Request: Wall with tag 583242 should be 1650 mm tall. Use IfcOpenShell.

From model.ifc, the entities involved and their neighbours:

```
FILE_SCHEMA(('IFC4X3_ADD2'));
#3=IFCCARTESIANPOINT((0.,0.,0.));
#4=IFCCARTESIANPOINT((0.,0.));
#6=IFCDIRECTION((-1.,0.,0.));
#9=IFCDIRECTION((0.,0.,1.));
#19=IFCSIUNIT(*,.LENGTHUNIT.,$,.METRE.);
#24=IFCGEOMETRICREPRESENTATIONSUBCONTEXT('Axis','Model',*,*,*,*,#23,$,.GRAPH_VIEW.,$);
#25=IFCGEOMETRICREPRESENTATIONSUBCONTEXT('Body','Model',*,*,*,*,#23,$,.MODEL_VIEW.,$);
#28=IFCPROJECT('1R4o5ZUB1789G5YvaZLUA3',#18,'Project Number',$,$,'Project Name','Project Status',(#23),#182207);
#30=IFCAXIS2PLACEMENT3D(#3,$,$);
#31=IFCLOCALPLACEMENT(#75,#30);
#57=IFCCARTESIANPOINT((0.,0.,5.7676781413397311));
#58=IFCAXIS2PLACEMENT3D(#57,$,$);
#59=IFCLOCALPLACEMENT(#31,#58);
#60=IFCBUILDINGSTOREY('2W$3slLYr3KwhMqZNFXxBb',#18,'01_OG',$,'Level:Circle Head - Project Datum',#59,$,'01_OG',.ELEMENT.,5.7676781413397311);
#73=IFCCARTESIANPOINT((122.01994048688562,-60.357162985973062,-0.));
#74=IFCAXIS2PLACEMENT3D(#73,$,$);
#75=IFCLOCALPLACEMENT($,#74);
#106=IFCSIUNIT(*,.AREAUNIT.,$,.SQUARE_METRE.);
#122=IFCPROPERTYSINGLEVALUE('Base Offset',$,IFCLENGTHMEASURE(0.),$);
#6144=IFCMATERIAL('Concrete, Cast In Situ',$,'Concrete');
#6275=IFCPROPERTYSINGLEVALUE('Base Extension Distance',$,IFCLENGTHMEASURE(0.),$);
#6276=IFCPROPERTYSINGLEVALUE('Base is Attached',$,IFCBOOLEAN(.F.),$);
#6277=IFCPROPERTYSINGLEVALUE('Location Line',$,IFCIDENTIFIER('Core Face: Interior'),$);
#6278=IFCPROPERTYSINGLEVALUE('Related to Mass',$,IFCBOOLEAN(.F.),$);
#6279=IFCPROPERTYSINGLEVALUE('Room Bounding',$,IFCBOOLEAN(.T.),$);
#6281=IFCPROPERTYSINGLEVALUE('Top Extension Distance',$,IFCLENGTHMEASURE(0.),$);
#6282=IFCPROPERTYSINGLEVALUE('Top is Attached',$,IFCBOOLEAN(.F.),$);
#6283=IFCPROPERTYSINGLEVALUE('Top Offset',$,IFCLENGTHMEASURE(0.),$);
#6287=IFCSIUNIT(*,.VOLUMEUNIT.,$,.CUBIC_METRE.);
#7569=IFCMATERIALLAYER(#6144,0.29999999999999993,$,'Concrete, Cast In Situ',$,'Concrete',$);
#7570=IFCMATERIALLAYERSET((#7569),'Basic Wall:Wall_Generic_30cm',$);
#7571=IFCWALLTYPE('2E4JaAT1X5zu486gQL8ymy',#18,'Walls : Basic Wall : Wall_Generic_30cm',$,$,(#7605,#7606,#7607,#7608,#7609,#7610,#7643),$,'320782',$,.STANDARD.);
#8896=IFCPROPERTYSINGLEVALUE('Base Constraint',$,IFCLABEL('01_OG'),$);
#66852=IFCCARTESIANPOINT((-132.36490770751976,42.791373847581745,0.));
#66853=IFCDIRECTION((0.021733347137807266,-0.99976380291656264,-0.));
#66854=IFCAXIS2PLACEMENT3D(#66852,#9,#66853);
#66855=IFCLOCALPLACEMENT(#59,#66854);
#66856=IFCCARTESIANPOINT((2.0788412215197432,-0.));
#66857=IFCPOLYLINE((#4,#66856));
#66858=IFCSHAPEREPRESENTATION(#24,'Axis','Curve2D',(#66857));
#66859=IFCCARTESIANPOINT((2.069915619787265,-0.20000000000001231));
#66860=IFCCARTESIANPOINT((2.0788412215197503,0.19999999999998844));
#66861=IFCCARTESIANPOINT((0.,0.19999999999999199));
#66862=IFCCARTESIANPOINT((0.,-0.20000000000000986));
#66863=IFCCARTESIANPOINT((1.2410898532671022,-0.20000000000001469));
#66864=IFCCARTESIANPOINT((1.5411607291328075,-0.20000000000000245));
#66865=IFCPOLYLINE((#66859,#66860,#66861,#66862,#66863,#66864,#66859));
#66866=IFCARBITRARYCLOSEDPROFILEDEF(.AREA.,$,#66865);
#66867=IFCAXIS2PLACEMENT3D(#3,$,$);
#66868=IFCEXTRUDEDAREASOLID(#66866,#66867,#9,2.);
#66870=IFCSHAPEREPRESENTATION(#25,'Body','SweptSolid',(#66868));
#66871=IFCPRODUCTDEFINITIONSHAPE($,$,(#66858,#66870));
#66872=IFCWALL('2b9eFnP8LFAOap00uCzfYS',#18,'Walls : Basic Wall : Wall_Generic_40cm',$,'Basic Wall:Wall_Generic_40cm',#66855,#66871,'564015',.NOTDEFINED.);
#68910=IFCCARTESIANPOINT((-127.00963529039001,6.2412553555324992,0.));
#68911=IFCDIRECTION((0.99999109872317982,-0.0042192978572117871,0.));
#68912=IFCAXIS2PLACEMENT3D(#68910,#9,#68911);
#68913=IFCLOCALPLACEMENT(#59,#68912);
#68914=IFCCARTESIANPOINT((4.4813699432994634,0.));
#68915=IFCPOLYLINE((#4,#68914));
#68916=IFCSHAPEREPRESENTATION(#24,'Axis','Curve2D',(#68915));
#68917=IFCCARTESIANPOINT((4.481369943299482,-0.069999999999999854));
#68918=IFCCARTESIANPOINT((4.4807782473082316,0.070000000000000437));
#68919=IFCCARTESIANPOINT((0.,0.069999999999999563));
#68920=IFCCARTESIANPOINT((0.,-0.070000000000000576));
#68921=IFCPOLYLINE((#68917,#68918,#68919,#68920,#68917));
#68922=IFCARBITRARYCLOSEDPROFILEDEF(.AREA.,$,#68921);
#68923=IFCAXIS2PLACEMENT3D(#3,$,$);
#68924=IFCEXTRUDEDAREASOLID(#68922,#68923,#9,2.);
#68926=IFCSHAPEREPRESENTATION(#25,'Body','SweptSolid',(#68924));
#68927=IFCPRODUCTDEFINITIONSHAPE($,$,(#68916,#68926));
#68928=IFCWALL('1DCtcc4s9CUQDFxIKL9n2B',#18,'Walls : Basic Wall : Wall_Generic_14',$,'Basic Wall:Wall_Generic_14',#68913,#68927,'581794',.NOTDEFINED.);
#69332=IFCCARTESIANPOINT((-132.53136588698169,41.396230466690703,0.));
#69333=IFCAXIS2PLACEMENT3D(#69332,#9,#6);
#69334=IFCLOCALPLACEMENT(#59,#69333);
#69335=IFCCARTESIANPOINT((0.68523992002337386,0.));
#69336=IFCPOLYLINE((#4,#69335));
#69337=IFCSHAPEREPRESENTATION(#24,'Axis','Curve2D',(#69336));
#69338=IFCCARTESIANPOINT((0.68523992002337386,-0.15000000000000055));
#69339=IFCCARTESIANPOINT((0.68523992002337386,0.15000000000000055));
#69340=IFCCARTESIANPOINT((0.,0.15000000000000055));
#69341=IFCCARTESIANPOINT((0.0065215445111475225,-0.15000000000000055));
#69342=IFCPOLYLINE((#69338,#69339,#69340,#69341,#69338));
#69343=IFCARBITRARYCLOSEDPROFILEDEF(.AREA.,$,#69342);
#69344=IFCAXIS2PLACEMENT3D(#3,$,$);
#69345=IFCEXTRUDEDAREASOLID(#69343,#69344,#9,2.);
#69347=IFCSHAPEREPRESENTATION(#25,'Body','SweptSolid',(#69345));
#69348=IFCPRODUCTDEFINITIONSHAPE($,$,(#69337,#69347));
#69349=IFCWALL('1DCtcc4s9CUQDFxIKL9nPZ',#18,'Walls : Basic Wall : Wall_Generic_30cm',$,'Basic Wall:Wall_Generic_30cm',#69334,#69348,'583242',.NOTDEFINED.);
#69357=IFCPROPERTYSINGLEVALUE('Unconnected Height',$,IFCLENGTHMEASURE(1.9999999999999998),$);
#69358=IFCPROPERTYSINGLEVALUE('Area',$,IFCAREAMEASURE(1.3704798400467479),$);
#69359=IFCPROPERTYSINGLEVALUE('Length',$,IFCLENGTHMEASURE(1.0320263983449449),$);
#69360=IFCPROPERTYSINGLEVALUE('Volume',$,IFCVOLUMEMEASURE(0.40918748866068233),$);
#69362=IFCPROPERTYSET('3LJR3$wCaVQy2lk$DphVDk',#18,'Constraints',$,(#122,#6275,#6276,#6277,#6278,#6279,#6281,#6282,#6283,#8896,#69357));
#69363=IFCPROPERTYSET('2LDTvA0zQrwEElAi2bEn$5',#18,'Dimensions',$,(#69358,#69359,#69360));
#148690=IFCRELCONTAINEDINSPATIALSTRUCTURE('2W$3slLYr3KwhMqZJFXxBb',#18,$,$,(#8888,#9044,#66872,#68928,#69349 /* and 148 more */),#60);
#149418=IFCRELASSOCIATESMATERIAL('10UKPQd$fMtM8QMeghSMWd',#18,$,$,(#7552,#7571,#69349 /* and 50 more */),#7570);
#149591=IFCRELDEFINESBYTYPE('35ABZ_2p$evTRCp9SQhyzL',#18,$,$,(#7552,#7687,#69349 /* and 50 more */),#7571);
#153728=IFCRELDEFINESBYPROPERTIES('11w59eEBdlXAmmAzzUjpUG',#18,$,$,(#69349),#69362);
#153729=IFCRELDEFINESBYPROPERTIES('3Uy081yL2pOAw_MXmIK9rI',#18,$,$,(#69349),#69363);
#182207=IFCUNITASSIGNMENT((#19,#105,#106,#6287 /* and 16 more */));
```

```python
import ifcopenshell
import ifcopenshell.api.pset
import ifcopenshell.geom
import ifcopenshell.util.element
import ifcopenshell.util.representation
import ifcopenshell.util.shape
import ifcopenshell.util.unit

model = ifcopenshell.open("model.ifc")
area_scale = ifcopenshell.util.unit.calculate_unit_scale(model, "AREAUNIT")
volume_scale = ifcopenshell.util.unit.calculate_unit_scale(model, "VOLUMEUNIT")
settings = ifcopenshell.geom.settings()


def volume(element):
    """Net volume in cubic metres, openings subtracted."""
    shape = ifcopenshell.geom.create_shape(settings, element)
    return ifcopenshell.util.shape.get_volume(shape.geometry)


wall = model.by_guid("1DCtcc4s9CUQDFxIKL9nPZ")
before = volume(wall)

body = ifcopenshell.util.representation.get_representation(wall, "Model", "Body")
solid = body.Items[0]
old_height = solid.Depth
solid.Depth = 1.65
after = volume(wall)
thickness = 0.3  # wall thickness in metres

# Update the stored height, areas and volumes.
pset = model.by_id(ifcopenshell.util.element.get_pset(wall, "Constraints", should_inherit=False)["id"])
ifcopenshell.api.pset.edit_pset(model, pset=pset, properties={
    "Unconnected Height": model.create_entity("IfcLengthMeasure", solid.Depth),
})
pset = model.by_id(ifcopenshell.util.element.get_pset(wall, "Dimensions", should_inherit=False)["id"])
ifcopenshell.api.pset.edit_pset(model, pset=pset, properties={
    "Area": model.create_entity("IfcAreaMeasure", after / thickness / area_scale),
    "Volume": model.create_entity("IfcVolumeMeasure", after / volume_scale),
})

print(f"height {old_height:g} -> {solid.Depth:g}, volume {before:.3f} -> {after:.3f} m3")

model.write("model_edited.ifc")
```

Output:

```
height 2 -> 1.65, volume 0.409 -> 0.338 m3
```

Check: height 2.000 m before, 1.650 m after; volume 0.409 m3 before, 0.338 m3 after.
